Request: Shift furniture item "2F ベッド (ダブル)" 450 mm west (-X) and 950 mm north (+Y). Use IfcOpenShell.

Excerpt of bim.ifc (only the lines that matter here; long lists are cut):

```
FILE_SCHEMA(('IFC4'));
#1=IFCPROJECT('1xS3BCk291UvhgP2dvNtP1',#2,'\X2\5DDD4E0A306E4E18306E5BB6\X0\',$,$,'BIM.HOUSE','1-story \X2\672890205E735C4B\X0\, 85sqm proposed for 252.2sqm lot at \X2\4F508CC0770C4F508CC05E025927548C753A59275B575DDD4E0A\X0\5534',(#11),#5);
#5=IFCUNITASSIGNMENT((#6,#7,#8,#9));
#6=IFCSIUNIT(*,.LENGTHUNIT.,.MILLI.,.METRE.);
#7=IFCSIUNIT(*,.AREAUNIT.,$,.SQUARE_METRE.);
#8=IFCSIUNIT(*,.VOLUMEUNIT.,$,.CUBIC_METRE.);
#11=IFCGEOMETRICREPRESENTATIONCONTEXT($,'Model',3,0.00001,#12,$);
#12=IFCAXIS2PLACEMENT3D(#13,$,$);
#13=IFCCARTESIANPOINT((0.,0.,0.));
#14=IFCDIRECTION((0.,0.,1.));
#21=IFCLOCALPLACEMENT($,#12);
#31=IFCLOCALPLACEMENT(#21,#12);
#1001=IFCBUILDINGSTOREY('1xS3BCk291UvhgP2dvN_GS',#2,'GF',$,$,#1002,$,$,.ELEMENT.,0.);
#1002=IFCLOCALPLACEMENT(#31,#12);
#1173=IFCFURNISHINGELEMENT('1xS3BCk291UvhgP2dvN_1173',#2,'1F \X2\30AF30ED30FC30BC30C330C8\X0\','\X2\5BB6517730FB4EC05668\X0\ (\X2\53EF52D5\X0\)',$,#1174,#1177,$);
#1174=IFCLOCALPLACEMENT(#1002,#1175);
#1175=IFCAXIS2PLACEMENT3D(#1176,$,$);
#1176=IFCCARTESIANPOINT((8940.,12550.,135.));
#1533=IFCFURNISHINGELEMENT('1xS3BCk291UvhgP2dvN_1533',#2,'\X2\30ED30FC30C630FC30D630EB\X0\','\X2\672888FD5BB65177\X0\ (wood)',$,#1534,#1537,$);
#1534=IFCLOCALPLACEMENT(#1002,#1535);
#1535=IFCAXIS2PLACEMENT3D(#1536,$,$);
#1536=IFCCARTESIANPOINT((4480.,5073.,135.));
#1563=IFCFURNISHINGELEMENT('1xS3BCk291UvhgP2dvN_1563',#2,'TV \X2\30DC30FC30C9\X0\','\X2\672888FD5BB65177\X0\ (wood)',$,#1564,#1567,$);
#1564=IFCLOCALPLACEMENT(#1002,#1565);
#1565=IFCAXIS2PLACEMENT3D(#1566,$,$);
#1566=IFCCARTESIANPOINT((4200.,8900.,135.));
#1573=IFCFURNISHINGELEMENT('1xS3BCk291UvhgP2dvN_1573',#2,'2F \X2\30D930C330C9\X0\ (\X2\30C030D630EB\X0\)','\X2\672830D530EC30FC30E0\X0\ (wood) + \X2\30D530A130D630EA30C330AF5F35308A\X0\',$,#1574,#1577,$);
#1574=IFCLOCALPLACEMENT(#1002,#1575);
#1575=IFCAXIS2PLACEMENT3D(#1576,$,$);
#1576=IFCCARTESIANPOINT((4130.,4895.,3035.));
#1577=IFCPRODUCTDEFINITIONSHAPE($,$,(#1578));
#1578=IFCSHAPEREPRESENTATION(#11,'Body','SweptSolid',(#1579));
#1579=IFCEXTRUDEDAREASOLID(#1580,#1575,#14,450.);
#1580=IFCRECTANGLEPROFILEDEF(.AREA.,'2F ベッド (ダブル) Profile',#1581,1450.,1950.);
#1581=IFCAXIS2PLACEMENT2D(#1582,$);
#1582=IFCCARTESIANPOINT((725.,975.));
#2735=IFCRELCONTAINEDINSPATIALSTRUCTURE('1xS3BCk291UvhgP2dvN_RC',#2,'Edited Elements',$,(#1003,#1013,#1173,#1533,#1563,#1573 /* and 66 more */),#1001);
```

```python
import ifcopenshell
import ifcopenshell.api.geometry
import ifcopenshell.util.placement

model = ifcopenshell.open("bim.ifc")

item = model.by_guid("1xS3BCk291UvhgP2dvN_1573")
matrix = ifcopenshell.util.placement.get_local_placement(item.ObjectPlacement)
matrix[0, 3] -= 450.0
matrix[1, 3] += 950.0
ifcopenshell.api.geometry.edit_object_placement(model, product=item, matrix=matrix, is_si=False)

print(ifcopenshell.util.placement.get_local_placement(item.ObjectPlacement).round(3) + 0.0)

model.write("bim_v2.ifc")
```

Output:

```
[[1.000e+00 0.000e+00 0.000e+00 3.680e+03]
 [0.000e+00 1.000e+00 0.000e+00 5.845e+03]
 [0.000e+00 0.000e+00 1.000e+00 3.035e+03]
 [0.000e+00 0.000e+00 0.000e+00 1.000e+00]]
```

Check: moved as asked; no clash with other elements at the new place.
